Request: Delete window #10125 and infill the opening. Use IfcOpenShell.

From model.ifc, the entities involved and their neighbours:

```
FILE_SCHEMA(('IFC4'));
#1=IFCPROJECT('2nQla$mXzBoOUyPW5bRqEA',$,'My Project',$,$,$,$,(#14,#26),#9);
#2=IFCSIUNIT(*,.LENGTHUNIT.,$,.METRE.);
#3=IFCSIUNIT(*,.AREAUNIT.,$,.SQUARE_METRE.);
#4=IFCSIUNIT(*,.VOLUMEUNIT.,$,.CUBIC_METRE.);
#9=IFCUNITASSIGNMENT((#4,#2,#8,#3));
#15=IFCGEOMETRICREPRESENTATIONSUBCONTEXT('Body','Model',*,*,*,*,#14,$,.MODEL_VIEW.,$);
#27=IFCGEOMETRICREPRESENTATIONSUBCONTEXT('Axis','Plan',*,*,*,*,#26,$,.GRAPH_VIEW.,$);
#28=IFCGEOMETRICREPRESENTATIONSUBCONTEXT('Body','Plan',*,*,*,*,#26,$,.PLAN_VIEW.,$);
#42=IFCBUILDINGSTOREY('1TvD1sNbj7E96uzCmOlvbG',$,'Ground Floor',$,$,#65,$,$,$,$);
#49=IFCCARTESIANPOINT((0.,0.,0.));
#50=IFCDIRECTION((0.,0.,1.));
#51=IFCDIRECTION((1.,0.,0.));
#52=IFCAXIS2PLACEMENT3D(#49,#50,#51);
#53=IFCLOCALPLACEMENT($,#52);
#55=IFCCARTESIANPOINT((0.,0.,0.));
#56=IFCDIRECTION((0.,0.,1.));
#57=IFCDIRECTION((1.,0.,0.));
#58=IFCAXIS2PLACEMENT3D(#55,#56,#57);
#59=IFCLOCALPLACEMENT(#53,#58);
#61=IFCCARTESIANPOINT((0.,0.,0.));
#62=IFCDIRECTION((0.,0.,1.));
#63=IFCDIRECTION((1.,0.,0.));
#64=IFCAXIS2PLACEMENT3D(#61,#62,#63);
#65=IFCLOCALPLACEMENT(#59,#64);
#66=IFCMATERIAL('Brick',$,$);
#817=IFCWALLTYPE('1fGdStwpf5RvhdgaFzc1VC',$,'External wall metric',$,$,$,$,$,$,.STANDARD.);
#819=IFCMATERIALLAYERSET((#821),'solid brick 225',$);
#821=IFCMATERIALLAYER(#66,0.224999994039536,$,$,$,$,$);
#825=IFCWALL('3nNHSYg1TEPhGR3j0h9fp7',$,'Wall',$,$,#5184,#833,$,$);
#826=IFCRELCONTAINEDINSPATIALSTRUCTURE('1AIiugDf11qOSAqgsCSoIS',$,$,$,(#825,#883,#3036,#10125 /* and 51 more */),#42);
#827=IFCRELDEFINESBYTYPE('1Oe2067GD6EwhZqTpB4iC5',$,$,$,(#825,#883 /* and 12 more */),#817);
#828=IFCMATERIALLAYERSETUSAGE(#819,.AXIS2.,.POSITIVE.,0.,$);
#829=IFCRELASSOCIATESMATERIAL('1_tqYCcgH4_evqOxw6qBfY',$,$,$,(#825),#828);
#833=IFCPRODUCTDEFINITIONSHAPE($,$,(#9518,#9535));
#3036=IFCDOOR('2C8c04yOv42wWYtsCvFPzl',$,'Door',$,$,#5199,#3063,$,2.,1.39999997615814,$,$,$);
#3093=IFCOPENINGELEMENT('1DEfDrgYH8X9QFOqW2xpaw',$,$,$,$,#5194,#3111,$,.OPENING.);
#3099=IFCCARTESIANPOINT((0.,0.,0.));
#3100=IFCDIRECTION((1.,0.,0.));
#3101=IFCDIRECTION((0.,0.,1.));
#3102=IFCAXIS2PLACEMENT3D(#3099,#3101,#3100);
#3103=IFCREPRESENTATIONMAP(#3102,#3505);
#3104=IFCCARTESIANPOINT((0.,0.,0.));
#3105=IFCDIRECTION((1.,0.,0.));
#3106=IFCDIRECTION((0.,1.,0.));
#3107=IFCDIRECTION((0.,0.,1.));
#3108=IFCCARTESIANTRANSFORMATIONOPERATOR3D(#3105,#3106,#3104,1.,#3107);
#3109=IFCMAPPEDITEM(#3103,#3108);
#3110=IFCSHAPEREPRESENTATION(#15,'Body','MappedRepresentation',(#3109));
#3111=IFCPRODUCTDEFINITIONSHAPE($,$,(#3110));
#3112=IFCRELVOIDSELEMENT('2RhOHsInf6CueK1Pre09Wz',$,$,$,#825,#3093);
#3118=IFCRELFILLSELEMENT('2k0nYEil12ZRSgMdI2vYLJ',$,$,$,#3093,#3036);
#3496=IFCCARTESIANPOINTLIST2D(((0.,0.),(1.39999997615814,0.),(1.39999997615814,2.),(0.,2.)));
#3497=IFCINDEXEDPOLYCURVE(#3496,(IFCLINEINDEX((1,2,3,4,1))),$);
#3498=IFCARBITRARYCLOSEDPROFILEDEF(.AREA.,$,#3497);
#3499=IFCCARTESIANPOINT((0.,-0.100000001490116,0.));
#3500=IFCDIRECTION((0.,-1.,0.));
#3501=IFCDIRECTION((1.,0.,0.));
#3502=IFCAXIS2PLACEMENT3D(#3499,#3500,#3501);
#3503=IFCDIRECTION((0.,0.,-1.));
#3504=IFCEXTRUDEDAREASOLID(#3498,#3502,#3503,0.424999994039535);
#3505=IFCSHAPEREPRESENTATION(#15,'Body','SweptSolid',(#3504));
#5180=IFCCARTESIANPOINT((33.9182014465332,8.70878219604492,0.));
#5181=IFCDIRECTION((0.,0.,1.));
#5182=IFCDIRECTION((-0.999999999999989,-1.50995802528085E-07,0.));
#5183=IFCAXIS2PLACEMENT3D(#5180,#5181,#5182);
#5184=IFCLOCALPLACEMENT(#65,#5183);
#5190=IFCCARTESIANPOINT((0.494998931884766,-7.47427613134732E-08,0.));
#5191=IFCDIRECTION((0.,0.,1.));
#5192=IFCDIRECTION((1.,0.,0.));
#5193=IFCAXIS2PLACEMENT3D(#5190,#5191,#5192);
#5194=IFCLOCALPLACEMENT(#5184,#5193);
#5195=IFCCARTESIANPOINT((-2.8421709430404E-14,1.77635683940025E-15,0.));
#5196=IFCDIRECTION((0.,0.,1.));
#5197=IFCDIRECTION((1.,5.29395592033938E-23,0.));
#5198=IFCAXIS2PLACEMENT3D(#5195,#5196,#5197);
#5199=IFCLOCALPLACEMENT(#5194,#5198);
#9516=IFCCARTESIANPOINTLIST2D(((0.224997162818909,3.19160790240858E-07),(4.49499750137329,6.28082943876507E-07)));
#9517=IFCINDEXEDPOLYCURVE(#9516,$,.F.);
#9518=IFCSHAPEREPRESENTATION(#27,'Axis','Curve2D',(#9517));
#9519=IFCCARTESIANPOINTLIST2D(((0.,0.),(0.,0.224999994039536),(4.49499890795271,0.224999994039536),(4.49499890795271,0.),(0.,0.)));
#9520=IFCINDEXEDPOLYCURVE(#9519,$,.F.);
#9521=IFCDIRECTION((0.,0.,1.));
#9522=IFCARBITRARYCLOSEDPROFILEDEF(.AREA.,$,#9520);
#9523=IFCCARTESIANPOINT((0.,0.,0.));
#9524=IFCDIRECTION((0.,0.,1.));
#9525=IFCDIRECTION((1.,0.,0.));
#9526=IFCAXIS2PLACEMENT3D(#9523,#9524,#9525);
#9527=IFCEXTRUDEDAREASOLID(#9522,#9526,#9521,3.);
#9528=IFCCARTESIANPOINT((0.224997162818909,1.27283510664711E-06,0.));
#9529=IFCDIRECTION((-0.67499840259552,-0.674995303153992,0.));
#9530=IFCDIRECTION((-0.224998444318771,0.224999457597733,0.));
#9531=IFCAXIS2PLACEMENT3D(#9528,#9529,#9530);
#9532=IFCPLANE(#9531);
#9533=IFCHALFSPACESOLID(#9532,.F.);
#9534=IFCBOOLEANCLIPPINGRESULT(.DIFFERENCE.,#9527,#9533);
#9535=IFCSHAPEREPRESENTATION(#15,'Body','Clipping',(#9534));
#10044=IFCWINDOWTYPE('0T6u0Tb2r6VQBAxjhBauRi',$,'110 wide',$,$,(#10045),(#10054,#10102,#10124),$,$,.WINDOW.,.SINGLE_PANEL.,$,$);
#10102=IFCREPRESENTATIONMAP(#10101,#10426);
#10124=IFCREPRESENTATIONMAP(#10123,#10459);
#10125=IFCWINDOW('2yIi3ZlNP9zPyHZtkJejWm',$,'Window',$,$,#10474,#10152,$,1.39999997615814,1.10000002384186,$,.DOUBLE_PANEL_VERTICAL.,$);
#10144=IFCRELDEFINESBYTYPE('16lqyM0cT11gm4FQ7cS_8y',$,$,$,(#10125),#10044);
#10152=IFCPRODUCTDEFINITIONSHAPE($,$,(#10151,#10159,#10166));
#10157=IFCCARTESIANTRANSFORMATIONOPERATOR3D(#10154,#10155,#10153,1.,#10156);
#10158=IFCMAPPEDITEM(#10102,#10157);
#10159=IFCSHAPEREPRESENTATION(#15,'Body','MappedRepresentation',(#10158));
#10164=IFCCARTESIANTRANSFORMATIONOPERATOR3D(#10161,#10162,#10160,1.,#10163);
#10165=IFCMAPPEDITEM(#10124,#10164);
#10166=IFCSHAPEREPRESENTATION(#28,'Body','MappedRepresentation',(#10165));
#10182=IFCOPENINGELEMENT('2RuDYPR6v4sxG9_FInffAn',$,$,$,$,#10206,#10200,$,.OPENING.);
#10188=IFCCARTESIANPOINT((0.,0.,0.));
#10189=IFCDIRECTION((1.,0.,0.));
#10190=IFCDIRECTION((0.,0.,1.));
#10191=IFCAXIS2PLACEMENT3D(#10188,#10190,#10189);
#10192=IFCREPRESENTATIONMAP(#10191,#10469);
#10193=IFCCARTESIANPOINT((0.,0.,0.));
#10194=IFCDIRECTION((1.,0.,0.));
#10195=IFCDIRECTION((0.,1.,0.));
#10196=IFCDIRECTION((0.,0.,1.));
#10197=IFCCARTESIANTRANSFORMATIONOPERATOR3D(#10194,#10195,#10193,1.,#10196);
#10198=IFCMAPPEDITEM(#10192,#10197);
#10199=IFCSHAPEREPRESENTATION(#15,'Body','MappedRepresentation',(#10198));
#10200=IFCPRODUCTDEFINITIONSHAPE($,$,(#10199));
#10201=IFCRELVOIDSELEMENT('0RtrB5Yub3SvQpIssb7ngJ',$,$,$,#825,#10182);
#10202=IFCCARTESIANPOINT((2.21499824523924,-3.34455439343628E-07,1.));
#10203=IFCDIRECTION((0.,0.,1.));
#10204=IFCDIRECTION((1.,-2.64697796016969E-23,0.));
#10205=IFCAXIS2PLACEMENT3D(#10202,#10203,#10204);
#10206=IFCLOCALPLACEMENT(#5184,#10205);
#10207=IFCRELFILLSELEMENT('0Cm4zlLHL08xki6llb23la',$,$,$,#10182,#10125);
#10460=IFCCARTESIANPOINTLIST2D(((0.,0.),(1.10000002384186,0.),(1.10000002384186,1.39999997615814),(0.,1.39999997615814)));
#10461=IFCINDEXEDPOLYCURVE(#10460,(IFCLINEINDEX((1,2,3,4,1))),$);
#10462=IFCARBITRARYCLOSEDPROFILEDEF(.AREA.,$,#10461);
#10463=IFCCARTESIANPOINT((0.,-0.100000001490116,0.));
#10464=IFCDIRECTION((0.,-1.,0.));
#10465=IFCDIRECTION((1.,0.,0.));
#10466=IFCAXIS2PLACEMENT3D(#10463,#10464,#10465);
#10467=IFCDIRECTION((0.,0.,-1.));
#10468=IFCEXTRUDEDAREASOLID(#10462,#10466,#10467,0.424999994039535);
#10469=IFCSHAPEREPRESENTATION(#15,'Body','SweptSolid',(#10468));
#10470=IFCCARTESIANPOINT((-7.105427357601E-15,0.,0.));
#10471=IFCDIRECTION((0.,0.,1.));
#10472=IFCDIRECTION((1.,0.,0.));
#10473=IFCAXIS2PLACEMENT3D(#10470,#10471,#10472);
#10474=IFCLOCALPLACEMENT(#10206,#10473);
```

```python
import ifcopenshell
import ifcopenshell.api.feature
import ifcopenshell.api.root
import ifcopenshell.geom
import ifcopenshell.util.shape

model = ifcopenshell.open("model.ifc")
settings = ifcopenshell.geom.settings()


def volume(element):
    """Net volume in cubic metres, openings subtracted."""
    shape = ifcopenshell.geom.create_shape(settings, element)
    return ifcopenshell.util.shape.get_volume(shape.geometry)


window = model.by_id(10125)
opening = window.FillsVoids[0].RelatingOpeningElement
wall = opening.VoidsElements[0].RelatingBuildingElement
before = volume(wall)

ifcopenshell.api.root.remove_product(model, product=window)
ifcopenshell.api.feature.remove_feature(model, feature=opening)

after = volume(wall)

print(f"wall volume {before:.3f} -> {after:.3f} m3")

model.write("model_edited.ifc")
```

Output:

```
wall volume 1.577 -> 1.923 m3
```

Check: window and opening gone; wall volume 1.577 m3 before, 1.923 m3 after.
